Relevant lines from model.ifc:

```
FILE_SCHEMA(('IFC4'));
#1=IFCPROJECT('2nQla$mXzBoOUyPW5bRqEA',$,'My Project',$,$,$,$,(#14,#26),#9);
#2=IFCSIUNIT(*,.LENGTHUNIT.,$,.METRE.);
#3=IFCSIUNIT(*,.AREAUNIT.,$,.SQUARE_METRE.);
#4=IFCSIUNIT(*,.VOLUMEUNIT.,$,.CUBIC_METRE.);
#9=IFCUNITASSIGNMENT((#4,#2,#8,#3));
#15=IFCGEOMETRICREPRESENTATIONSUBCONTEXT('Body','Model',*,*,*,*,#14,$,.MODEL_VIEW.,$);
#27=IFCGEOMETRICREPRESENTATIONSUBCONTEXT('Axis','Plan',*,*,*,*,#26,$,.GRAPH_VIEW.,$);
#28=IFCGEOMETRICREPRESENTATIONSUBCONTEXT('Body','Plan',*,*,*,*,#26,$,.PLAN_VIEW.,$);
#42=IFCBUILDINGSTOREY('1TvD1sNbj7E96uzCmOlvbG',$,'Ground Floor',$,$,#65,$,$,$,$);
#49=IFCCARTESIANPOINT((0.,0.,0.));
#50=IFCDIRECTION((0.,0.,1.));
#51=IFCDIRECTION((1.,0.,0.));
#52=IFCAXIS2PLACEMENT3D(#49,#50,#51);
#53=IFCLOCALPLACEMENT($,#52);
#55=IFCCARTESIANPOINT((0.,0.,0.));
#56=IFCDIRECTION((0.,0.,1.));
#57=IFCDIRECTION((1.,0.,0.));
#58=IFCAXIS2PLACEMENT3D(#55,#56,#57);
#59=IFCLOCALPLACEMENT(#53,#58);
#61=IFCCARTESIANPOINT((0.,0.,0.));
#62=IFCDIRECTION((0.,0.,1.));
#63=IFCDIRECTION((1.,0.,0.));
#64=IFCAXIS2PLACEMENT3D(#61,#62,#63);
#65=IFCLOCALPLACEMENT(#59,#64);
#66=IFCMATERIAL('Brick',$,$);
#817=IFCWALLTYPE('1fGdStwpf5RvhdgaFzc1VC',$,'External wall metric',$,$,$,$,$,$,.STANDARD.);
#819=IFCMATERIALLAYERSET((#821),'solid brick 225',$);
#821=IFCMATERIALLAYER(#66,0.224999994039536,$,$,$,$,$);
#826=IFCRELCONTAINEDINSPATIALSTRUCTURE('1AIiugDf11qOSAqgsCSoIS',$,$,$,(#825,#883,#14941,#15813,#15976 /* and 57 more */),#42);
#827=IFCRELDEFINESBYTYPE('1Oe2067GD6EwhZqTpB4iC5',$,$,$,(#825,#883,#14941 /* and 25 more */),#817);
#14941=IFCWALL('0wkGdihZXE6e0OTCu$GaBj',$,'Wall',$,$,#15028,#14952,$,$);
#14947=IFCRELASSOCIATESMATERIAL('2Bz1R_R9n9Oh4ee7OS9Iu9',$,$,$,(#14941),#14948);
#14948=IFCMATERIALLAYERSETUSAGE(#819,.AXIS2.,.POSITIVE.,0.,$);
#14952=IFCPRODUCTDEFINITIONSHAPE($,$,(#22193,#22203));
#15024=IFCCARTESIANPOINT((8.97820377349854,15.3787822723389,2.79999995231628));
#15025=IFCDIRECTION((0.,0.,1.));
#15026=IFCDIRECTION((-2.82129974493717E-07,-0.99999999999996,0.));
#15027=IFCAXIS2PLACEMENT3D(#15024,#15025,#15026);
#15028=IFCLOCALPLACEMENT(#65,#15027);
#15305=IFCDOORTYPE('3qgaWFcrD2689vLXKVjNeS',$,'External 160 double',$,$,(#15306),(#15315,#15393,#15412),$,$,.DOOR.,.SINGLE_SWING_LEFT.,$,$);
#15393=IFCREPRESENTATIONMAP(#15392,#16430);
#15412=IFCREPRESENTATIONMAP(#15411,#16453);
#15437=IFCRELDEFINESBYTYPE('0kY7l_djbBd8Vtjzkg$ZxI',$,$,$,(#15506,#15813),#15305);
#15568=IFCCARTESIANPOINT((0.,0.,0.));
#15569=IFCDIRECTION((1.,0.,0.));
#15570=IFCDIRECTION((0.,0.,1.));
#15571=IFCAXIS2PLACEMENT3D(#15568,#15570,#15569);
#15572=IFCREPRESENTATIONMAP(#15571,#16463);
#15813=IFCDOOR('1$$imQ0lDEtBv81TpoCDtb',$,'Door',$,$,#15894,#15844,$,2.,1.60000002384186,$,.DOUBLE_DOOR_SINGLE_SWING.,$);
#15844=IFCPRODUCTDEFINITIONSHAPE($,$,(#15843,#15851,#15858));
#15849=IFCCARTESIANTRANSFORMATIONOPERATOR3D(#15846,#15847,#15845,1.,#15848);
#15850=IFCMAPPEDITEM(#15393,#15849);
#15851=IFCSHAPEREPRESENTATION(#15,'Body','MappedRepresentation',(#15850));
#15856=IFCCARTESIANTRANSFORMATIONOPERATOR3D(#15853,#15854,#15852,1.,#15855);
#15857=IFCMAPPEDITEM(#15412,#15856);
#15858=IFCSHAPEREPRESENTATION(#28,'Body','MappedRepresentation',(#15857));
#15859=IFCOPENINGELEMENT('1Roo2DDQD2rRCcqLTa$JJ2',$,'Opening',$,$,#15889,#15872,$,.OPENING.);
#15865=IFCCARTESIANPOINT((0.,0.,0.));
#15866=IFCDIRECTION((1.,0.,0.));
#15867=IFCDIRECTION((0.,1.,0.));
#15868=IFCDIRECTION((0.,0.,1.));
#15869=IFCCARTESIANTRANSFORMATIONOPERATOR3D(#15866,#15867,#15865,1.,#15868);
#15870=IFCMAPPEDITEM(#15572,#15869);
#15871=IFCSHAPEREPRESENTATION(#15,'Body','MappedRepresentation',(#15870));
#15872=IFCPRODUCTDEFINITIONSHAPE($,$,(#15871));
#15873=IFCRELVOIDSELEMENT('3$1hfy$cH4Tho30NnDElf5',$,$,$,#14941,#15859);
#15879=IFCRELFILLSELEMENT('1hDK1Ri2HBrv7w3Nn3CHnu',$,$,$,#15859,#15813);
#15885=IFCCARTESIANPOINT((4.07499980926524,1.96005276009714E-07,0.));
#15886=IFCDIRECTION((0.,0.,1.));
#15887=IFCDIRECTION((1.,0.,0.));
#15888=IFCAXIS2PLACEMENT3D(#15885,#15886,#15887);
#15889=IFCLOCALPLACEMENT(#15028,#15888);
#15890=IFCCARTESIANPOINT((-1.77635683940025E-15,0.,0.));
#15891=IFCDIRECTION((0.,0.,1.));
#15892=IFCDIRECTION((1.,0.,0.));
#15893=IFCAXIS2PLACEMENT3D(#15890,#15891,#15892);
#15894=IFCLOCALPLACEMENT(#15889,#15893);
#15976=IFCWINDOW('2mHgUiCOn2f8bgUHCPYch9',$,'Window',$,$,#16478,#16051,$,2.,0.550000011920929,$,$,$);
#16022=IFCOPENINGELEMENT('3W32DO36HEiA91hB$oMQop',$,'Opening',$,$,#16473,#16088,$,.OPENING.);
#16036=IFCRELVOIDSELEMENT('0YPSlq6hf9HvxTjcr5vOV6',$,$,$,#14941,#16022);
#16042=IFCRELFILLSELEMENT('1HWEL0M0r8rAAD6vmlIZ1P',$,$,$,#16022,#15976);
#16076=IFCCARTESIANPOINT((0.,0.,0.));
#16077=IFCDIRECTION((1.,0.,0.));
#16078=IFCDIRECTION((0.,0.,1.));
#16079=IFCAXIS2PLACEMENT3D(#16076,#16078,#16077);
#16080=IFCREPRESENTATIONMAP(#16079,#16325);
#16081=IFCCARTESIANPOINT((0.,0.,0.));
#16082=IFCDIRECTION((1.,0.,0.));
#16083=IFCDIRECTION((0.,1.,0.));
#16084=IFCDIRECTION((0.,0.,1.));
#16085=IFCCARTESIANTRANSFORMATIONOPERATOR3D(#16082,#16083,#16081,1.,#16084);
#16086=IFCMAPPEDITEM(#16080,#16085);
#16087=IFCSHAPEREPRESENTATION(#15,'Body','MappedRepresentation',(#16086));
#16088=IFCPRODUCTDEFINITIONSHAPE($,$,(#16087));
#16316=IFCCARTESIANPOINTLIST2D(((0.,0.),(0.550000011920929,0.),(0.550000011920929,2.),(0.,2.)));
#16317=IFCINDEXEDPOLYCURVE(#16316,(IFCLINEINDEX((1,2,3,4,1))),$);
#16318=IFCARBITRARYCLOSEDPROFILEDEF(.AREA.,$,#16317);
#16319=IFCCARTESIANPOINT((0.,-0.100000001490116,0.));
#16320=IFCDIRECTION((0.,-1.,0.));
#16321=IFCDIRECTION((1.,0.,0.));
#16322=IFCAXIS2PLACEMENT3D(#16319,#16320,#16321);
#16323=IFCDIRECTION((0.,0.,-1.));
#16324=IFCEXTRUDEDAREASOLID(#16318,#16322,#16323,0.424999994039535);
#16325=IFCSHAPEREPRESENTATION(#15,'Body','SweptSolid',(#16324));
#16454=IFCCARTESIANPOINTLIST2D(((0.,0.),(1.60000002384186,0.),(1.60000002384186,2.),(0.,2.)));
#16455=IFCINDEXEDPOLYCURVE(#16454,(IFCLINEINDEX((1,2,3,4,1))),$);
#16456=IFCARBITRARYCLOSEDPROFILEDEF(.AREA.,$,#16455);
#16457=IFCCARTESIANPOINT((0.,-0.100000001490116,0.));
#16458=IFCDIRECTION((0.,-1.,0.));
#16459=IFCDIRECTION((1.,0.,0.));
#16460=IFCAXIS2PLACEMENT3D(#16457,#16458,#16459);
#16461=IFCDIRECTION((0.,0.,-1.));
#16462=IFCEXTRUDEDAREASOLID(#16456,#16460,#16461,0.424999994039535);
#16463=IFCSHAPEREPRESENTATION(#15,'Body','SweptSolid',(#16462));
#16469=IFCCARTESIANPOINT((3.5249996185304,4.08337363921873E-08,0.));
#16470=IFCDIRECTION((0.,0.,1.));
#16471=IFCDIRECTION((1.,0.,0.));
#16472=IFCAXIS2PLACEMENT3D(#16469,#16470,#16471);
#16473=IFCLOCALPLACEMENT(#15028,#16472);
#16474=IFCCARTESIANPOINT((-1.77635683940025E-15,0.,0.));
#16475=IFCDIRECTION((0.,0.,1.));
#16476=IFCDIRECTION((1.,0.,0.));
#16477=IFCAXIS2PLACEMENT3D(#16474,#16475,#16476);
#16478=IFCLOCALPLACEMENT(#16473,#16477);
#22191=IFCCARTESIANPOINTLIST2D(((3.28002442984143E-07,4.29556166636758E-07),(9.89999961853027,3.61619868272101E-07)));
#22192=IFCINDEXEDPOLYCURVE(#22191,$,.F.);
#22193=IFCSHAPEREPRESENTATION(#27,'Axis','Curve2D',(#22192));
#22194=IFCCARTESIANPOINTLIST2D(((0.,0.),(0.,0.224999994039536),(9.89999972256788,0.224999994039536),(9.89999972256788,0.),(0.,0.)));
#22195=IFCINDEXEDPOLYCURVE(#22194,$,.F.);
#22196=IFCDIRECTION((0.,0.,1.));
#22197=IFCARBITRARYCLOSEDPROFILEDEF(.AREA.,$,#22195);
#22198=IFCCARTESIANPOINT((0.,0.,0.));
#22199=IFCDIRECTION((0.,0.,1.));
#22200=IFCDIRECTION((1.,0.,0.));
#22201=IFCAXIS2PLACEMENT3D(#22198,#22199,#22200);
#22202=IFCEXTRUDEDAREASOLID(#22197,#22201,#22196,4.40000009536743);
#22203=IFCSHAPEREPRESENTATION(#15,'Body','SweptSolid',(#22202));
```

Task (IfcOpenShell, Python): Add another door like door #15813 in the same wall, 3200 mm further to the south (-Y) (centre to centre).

```python
import ifcopenshell
import ifcopenshell.api.feature
import ifcopenshell.api.geometry
import ifcopenshell.api.root
import ifcopenshell.geom
import ifcopenshell.util.element
import ifcopenshell.util.placement
import ifcopenshell.util.shape

model = ifcopenshell.open("model.ifc")
settings = ifcopenshell.geom.settings()


def volume(element):
    """Net volume in cubic metres, openings subtracted."""
    shape = ifcopenshell.geom.create_shape(settings, element)
    return ifcopenshell.util.shape.get_volume(shape.geometry)


door = model.by_id(15813)
opening = door.FillsVoids[0].RelatingOpeningElement
wall = opening.VoidsElements[0].RelatingBuildingElement
before = volume(wall)
shift = ifcopenshell.util.placement.get_local_placement(wall.ObjectPlacement)[:3, 0] * 3.2

# copy_class copies the void relationship, type, container and properties, but no geometry.
new_opening = ifcopenshell.api.root.copy_class(model, product=opening)
new_opening.Representation = ifcopenshell.util.element.copy_deep(
    model, opening.Representation, exclude=["IfcGeometricRepresentationContext", "IfcRepresentationMap"]
)
new_door = ifcopenshell.api.root.copy_class(model, product=door)
new_door.Representation = ifcopenshell.util.element.copy_deep(
    model, door.Representation, exclude=["IfcGeometricRepresentationContext", "IfcRepresentationMap"]
)
ifcopenshell.api.feature.add_filling(model, opening=new_opening, element=new_door)

for old, new in ((opening, new_opening), (door, new_door)):
    matrix = ifcopenshell.util.placement.get_local_placement(old.ObjectPlacement)
    matrix[:3, 3] += shift
    ifcopenshell.api.geometry.edit_object_placement(model, product=new, matrix=matrix, is_si=False)

after = volume(wall)

print(f"wall volume {before:.3f} -> {after:.3f} m3")

model.write("model_updated.ifc")
```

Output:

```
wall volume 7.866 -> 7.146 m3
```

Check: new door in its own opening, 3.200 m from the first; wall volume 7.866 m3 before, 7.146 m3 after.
